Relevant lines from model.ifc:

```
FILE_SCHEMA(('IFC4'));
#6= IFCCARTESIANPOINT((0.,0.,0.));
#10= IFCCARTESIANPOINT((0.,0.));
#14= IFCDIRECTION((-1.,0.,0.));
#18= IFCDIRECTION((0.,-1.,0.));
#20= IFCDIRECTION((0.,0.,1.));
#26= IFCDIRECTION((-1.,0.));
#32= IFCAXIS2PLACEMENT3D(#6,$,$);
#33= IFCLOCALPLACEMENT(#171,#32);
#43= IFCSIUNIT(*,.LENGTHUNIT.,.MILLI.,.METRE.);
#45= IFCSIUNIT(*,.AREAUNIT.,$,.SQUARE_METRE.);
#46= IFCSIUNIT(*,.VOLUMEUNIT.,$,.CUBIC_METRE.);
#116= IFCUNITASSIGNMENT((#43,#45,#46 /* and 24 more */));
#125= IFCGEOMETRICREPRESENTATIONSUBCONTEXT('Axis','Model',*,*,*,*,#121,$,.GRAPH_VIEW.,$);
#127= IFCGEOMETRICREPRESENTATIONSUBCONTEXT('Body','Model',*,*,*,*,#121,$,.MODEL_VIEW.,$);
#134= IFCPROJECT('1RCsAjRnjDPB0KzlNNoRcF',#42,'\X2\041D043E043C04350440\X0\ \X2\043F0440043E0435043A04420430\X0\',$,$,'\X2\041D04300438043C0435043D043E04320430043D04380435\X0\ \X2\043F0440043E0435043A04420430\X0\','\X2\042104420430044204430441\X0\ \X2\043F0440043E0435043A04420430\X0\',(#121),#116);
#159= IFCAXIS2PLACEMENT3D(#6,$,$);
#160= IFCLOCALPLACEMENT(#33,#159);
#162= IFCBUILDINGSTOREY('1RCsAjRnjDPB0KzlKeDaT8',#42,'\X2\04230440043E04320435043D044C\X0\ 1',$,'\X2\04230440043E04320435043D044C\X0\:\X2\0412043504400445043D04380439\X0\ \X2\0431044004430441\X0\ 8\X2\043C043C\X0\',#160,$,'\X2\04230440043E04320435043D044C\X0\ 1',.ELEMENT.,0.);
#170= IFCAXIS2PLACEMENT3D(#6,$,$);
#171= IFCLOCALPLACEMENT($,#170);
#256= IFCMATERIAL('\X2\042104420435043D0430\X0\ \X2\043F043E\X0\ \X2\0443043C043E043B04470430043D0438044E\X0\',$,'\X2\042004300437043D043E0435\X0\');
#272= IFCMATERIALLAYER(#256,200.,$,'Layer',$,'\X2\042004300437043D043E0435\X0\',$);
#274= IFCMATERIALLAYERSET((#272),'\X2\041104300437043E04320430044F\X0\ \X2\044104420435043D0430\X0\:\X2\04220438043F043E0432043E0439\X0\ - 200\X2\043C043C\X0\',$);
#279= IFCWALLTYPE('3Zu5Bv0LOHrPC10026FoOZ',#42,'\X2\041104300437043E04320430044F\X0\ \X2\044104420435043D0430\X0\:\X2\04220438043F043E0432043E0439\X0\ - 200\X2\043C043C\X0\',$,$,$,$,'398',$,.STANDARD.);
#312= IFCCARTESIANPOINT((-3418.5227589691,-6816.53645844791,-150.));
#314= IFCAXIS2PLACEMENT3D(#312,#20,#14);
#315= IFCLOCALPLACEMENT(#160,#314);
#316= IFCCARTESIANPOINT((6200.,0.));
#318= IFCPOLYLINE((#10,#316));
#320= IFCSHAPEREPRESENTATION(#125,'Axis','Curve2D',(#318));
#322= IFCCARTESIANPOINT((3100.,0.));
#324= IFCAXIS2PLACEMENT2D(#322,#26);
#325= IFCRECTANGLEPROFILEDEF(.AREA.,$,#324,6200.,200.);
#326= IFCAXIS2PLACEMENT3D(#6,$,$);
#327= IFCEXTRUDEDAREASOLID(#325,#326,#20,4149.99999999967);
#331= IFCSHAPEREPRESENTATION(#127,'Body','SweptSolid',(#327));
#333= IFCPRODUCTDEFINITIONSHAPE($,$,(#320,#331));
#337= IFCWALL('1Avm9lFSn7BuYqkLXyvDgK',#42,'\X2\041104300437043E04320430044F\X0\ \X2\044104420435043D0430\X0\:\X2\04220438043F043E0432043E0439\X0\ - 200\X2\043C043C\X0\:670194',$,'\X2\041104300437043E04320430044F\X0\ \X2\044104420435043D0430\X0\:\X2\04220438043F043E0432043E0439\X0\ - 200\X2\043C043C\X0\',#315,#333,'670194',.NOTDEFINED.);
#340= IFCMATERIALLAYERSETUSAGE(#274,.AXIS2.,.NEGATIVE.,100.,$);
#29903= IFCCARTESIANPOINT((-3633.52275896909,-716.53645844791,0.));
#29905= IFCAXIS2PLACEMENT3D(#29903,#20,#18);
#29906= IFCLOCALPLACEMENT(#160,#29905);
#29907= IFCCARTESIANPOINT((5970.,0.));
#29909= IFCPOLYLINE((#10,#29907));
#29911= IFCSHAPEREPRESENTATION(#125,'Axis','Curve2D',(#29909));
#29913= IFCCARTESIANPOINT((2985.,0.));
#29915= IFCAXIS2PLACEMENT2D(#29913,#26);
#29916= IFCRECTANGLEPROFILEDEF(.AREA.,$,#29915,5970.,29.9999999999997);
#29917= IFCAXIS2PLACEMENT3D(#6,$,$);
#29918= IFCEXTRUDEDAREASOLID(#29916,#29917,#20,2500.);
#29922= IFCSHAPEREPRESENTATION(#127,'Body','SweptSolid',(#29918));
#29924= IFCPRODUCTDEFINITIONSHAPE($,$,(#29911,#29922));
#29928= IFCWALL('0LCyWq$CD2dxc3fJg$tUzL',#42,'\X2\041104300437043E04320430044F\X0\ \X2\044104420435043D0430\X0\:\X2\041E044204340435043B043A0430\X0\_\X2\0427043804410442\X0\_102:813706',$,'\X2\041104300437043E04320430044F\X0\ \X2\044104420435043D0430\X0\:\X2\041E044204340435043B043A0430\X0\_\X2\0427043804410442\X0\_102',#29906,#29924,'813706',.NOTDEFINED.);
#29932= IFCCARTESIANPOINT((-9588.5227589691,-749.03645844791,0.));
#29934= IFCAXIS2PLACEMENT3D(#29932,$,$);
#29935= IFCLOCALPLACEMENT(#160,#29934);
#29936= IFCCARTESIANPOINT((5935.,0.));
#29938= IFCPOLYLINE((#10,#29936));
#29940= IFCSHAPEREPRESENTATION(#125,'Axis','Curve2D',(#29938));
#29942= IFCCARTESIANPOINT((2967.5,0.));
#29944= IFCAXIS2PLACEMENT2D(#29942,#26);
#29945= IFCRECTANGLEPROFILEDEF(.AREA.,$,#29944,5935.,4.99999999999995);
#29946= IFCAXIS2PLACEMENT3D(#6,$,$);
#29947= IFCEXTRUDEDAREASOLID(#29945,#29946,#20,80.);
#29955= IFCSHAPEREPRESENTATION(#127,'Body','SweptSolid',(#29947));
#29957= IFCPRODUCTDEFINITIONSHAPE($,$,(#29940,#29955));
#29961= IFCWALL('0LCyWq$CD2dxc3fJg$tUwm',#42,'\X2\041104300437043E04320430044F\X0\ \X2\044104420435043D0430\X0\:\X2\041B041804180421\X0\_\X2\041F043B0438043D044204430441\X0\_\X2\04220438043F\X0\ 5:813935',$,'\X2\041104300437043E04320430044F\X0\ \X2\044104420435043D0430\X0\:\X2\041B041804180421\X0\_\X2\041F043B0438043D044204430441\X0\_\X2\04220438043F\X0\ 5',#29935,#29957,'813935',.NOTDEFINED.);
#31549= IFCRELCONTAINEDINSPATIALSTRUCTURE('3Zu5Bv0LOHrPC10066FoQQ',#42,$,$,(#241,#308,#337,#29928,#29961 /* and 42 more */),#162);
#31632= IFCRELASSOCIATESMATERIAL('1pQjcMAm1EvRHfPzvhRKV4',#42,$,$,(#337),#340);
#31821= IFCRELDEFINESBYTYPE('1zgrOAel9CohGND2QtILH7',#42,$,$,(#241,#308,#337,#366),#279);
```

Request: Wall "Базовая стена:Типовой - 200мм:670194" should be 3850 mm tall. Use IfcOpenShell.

```python
import ifcopenshell
import ifcopenshell.geom
import ifcopenshell.util.representation
import ifcopenshell.util.shape

model = ifcopenshell.open("model.ifc")
settings = ifcopenshell.geom.settings()


def volume(element):
    """Net volume in cubic metres, openings subtracted."""
    shape = ifcopenshell.geom.create_shape(settings, element)
    return ifcopenshell.util.shape.get_volume(shape.geometry)


wall = model.by_id(337)
before = volume(wall)

body = ifcopenshell.util.representation.get_representation(wall, "Model", "Body")
solid = body.Items[0]
old_height = solid.Depth
solid.Depth = 3850.0
after = volume(wall)

print(f"height {old_height:g} -> {solid.Depth:g}, volume {before:.3f} -> {after:.3f} m3")

model.write("model-out.ifc")
```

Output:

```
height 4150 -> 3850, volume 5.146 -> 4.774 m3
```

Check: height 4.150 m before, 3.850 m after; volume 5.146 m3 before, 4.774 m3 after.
